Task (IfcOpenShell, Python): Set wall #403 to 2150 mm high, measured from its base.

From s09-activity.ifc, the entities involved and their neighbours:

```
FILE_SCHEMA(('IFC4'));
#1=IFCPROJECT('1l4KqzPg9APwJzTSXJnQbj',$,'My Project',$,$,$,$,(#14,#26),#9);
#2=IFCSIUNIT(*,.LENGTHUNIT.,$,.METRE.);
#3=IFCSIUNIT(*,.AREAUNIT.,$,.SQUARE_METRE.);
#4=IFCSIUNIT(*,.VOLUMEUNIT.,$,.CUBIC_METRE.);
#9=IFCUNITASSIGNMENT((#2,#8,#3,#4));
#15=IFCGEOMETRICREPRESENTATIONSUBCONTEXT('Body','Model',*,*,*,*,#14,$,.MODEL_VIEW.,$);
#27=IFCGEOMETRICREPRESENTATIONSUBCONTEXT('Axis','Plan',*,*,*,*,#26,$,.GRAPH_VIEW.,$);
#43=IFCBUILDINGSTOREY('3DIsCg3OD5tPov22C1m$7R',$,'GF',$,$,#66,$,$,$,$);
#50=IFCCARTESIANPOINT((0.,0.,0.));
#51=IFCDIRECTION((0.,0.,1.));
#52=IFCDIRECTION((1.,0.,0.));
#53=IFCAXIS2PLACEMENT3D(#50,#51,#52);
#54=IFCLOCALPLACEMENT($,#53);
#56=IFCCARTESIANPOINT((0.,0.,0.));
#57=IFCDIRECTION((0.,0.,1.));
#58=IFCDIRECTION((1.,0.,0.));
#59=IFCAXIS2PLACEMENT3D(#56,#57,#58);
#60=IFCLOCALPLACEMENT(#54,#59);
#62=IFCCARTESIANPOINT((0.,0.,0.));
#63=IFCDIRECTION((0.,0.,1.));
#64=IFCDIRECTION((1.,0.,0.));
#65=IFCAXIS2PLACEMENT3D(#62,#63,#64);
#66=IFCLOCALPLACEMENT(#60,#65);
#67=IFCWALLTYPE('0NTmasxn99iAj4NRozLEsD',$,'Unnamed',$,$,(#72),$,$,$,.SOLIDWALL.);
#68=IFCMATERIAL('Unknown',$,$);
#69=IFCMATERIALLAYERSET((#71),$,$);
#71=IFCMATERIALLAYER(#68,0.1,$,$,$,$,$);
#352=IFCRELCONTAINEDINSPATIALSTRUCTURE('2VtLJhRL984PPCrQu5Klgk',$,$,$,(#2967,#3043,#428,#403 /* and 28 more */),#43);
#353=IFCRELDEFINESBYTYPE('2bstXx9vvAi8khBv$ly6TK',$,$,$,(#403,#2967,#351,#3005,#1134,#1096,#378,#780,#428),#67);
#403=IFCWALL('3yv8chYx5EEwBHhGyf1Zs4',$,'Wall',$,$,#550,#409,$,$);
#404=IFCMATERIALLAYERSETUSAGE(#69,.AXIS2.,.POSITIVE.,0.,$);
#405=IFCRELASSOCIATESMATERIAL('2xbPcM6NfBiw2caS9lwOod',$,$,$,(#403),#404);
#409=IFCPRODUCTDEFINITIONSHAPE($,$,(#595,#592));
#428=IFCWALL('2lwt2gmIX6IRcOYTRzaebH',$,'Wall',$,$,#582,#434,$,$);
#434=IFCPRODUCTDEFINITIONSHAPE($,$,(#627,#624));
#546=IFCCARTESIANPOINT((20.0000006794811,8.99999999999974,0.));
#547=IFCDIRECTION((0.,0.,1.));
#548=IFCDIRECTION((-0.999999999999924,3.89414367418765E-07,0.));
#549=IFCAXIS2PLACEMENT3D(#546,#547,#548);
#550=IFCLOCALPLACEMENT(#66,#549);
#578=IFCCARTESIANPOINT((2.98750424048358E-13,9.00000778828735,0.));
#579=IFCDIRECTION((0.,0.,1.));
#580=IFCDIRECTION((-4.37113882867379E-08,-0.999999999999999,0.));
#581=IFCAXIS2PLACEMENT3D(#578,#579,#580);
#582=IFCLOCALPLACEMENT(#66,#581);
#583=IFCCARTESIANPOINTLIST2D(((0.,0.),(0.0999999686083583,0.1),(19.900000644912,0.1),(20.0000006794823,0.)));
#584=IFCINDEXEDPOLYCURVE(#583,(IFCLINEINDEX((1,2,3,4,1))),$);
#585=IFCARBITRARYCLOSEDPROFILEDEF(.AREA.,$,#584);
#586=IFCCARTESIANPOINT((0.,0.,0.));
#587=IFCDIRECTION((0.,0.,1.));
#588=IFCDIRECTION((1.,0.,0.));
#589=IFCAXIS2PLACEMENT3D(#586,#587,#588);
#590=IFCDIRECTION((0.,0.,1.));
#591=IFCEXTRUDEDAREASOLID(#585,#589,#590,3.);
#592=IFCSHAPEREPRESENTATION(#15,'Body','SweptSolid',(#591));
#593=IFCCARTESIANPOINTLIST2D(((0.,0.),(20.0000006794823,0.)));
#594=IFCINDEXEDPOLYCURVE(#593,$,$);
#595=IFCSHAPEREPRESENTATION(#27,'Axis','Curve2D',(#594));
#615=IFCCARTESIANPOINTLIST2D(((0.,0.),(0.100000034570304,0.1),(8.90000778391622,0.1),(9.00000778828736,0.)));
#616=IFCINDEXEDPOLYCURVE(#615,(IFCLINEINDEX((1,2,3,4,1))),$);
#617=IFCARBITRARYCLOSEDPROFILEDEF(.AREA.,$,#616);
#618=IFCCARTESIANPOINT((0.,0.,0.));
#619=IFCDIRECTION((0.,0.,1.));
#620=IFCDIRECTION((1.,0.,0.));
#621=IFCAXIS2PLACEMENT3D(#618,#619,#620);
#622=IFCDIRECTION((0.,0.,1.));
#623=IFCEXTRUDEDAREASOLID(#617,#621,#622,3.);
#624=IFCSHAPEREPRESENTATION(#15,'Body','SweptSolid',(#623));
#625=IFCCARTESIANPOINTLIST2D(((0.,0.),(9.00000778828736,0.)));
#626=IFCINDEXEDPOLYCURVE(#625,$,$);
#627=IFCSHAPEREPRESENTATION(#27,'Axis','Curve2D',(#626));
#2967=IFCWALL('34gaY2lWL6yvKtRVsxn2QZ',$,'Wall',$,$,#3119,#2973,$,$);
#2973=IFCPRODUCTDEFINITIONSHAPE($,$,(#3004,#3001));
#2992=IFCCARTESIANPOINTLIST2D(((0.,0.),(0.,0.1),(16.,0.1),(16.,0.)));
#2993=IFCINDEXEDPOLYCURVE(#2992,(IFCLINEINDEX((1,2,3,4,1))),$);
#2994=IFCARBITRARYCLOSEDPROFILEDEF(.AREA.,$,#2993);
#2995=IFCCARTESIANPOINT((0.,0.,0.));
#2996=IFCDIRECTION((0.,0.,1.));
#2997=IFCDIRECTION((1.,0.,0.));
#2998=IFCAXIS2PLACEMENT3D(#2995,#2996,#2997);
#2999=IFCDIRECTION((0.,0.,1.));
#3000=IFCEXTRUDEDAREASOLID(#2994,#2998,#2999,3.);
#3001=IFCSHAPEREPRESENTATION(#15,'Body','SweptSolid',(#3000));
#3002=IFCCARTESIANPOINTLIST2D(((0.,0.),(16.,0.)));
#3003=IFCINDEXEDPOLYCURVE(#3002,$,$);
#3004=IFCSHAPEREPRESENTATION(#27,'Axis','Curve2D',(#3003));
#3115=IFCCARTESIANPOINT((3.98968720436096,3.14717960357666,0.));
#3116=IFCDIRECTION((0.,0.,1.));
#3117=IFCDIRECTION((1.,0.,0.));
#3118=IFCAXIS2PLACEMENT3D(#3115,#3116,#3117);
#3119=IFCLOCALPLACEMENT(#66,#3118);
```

```python
import ifcopenshell
import ifcopenshell.geom
import ifcopenshell.util.representation
import ifcopenshell.util.shape

model = ifcopenshell.open("s09-activity.ifc")
settings = ifcopenshell.geom.settings()


def volume(element):
    """Net volume in cubic metres, openings subtracted."""
    shape = ifcopenshell.geom.create_shape(settings, element)
    return ifcopenshell.util.shape.get_volume(shape.geometry)


wall = model.by_id(403)
before = volume(wall)

body = ifcopenshell.util.representation.get_representation(wall, "Model", "Body")
solid = body.Items[0]
old_height = solid.Depth
solid.Depth = 2.15
after = volume(wall)

print(f"height {old_height:g} -> {solid.Depth:g}, volume {before:.3f} -> {after:.3f} m3")

model.write("s09-activity-out.ifc")
```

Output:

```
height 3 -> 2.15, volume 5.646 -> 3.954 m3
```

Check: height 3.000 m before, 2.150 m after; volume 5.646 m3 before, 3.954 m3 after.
